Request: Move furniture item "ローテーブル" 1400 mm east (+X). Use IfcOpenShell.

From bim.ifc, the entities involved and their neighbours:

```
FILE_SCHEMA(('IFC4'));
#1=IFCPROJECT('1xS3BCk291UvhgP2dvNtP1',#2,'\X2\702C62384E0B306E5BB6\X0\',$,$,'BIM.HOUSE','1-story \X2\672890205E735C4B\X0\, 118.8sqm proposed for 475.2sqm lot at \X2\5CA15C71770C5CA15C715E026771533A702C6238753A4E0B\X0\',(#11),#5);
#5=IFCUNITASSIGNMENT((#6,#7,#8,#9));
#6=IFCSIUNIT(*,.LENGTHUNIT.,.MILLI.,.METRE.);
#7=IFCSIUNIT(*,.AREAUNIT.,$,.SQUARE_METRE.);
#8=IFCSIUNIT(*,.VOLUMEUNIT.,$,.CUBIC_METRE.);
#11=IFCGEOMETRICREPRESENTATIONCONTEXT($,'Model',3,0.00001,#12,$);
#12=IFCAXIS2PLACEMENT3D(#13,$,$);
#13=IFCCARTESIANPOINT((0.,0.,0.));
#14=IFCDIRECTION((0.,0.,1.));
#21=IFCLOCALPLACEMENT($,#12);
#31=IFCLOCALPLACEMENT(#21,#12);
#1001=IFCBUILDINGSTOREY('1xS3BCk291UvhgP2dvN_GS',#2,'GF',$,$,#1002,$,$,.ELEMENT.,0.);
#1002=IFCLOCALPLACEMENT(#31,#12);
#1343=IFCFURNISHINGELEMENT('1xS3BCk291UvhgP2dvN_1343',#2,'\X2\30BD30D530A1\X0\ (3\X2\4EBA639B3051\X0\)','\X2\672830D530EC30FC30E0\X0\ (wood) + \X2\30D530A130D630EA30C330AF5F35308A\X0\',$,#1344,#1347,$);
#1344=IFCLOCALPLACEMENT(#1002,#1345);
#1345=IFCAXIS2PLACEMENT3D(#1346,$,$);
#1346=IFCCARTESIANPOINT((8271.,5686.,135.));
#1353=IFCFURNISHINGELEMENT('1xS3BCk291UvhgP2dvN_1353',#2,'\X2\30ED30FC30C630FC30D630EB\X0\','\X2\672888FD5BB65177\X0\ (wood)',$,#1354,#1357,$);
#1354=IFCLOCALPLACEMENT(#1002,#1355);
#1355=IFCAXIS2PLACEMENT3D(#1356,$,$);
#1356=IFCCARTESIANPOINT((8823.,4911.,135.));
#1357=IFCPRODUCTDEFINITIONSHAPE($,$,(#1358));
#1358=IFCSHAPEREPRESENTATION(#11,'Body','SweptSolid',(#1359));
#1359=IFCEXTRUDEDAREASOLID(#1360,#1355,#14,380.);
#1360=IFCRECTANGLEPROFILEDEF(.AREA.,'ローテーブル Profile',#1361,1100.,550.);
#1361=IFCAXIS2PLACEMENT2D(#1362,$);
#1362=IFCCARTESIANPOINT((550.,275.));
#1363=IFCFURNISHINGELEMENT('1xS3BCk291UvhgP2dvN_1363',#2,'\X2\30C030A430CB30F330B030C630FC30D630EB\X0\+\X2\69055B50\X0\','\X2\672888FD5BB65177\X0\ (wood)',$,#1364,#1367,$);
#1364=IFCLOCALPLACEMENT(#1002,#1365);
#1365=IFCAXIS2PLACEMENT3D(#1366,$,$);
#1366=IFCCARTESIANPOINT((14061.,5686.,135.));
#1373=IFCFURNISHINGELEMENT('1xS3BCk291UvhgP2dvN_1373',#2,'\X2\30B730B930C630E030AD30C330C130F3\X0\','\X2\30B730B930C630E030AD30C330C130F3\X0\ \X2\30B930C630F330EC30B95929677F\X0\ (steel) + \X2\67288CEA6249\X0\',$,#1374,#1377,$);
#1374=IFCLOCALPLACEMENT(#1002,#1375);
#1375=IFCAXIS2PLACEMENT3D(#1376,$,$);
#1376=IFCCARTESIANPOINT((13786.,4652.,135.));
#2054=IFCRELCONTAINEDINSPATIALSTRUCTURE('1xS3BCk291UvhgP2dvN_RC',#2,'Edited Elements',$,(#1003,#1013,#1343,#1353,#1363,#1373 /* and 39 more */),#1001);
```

```python
import ifcopenshell
import ifcopenshell.api.geometry
import ifcopenshell.util.placement

model = ifcopenshell.open("bim.ifc")

item = model.by_id(1353)
matrix = ifcopenshell.util.placement.get_local_placement(item.ObjectPlacement)
matrix[0, 3] += 1400.0
ifcopenshell.api.geometry.edit_object_placement(model, product=item, matrix=matrix, is_si=False)

print(ifcopenshell.util.placement.get_local_placement(item.ObjectPlacement).round(3) + 0.0)

model.write("bim_edited.ifc")
```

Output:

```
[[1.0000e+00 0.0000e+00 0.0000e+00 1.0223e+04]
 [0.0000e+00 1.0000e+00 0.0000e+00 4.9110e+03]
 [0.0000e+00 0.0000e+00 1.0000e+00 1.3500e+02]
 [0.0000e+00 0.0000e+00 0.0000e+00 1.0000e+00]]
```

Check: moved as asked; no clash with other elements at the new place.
